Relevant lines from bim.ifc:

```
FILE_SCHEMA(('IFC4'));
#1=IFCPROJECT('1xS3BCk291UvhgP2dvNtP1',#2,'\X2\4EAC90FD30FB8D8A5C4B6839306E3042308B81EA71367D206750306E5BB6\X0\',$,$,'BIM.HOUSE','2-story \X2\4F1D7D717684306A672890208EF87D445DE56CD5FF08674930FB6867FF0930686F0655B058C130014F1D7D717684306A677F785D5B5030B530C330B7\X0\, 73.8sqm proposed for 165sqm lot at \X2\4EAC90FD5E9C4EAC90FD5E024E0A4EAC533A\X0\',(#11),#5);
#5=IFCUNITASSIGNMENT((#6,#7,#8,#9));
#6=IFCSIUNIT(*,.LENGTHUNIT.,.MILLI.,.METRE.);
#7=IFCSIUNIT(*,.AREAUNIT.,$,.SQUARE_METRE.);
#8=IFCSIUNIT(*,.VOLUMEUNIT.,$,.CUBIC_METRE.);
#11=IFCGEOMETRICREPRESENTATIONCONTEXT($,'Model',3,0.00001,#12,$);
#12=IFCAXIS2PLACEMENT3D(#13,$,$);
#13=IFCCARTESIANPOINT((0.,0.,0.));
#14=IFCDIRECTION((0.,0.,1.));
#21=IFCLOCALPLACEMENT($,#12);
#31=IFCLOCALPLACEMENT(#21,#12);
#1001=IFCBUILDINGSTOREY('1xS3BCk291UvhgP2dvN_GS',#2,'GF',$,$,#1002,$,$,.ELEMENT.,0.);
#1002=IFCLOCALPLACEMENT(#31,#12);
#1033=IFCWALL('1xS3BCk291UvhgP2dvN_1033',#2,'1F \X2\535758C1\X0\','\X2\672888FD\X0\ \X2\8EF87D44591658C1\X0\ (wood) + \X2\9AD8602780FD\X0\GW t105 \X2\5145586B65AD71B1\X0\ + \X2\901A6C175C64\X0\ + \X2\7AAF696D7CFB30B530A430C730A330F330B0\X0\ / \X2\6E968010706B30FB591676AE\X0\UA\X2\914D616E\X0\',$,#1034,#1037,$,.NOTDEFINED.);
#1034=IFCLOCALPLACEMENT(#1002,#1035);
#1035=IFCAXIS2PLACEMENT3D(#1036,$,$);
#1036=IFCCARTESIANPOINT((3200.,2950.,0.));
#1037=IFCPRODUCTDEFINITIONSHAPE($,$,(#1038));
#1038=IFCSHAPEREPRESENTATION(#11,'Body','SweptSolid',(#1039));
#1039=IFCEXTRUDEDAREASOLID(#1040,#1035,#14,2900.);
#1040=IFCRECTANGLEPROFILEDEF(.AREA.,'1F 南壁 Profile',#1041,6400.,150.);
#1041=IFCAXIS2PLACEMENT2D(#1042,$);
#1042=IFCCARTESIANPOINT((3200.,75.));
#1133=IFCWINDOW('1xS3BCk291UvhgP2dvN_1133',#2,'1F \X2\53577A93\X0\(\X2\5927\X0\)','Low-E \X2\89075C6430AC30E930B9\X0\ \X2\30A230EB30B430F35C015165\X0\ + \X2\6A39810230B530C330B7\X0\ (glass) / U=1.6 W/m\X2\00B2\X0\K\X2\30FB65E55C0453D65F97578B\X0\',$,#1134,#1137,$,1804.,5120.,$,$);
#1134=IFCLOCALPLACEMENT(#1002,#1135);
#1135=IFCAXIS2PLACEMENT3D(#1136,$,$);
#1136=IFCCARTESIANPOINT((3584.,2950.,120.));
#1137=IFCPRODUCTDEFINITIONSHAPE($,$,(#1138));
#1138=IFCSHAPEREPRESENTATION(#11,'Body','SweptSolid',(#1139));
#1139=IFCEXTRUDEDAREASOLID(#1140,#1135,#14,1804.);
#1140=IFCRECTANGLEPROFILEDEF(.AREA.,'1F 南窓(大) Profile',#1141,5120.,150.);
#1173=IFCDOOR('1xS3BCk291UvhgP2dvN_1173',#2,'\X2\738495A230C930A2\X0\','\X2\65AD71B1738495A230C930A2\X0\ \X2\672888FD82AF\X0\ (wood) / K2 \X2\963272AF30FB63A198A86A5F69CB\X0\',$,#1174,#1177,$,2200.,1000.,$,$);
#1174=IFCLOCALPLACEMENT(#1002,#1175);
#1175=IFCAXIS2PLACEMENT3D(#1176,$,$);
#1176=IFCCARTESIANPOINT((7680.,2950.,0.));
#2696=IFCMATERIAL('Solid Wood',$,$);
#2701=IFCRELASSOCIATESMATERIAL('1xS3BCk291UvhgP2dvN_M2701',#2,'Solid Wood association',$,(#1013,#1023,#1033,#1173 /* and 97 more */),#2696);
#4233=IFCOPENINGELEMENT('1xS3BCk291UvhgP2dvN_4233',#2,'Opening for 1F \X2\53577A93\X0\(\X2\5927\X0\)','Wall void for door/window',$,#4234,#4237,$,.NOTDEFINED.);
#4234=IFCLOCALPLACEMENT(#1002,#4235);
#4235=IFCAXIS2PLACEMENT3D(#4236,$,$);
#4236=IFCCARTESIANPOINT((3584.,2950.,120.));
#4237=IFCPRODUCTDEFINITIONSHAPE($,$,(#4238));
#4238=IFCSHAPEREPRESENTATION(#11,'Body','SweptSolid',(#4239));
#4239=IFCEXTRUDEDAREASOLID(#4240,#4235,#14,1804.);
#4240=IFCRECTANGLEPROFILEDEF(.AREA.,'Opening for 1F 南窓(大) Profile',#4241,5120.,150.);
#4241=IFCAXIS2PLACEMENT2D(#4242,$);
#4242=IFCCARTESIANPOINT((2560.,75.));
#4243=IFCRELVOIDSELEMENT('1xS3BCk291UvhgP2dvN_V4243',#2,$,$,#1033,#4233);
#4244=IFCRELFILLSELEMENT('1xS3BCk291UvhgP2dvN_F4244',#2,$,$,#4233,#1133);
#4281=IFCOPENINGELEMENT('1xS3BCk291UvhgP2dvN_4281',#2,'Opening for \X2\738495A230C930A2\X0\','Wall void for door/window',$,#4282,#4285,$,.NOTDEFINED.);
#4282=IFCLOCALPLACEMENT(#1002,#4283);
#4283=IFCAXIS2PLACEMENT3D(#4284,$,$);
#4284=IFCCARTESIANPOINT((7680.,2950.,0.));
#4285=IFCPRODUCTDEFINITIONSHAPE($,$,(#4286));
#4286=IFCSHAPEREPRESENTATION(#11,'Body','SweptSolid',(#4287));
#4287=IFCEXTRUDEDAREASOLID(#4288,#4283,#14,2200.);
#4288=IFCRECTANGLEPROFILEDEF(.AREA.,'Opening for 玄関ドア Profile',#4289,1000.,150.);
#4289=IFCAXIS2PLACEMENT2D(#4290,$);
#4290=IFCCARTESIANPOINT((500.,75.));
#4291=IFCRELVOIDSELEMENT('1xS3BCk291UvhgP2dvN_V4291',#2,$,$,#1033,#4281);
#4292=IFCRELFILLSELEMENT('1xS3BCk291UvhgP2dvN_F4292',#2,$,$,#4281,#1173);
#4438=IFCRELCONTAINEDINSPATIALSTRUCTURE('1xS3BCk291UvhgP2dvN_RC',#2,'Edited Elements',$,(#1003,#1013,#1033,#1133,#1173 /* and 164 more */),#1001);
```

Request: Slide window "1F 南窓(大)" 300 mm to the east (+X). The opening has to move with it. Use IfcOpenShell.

```python
import ifcopenshell
import ifcopenshell.api.geometry
import ifcopenshell.util.placement

model = ifcopenshell.open("bim.ifc")

window = model.by_guid("1xS3BCk291UvhgP2dvN_1133")
opening = window.FillsVoids[0].RelatingOpeningElement
wall = opening.VoidsElements[0].RelatingBuildingElement

wall_matrix = ifcopenshell.util.placement.get_local_placement(wall.ObjectPlacement)
shift = wall_matrix[:3, 0] * 300.0
before = ifcopenshell.util.placement.get_local_placement(window.ObjectPlacement)[:3, 3].copy()

# The window is not placed relative to its opening, so move both.
for product in (opening, window):
    matrix = ifcopenshell.util.placement.get_local_placement(product.ObjectPlacement)
    matrix[:3, 3] += shift
    ifcopenshell.api.geometry.edit_object_placement(model, product=product, matrix=matrix, is_si=False)

after = ifcopenshell.util.placement.get_local_placement(window.ObjectPlacement)[:3, 3]
print("window moved by", (after - before).round(3) + 0.0)

model.write("bim_rev.ifc")
```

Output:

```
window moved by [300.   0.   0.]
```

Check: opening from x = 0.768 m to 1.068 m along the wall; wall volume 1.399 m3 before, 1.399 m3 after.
